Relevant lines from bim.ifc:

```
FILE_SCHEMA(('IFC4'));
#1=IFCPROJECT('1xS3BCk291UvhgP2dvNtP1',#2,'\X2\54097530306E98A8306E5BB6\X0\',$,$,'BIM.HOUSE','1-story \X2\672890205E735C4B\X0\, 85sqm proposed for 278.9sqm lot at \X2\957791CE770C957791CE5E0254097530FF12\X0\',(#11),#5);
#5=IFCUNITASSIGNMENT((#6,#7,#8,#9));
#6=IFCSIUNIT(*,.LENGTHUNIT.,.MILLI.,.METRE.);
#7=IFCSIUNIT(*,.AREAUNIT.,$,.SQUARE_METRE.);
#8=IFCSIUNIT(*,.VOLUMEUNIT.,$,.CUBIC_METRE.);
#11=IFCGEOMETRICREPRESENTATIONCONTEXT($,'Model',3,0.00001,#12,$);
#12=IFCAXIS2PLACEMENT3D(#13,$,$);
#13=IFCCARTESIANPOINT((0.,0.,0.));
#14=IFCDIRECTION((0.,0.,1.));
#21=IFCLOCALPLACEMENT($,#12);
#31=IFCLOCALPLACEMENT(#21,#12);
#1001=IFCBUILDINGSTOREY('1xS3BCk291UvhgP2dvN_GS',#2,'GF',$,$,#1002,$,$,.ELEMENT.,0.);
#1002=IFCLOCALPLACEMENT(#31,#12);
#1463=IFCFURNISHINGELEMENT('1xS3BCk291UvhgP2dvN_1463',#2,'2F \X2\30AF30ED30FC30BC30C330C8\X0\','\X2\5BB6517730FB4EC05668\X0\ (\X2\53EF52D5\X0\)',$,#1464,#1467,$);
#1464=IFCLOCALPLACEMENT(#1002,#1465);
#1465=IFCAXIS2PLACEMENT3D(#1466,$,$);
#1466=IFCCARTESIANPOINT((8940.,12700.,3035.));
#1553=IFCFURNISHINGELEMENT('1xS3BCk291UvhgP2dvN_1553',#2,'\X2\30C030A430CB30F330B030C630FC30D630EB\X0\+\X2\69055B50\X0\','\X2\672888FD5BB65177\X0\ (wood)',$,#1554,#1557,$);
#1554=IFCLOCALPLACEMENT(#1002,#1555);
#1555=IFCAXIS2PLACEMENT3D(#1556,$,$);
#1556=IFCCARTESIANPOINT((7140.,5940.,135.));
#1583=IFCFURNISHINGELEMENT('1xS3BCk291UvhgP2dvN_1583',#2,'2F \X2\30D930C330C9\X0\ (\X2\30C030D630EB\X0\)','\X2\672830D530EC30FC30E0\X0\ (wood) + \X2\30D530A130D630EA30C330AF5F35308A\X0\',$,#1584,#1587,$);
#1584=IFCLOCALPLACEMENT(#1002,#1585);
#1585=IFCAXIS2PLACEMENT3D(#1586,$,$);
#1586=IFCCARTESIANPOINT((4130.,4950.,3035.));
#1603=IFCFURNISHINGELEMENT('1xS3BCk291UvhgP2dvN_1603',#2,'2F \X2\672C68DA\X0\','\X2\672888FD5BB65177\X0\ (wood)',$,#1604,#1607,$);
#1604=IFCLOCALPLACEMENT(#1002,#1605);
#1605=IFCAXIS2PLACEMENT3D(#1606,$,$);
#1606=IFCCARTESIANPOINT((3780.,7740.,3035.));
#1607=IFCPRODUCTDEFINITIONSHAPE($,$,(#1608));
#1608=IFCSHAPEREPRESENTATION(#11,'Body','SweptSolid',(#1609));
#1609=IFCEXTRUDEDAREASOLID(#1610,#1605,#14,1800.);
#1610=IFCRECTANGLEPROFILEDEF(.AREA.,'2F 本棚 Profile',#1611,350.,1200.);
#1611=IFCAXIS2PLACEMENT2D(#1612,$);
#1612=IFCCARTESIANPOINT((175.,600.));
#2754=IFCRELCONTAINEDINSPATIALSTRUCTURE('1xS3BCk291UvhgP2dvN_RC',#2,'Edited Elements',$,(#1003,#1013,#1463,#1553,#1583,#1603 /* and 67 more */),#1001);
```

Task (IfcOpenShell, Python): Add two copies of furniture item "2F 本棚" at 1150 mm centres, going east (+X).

```python
import numpy as np
import ifcopenshell
import ifcopenshell.api.geometry
import ifcopenshell.api.root
import ifcopenshell.util.element
import ifcopenshell.util.placement
import ifcopenshell.util.unit

model = ifcopenshell.open("bim.ifc")
unit_scale = ifcopenshell.util.unit.calculate_unit_scale(model)


def reuse_history(source, copy):
    """copy_class also copies each property set's owner history, people and application; keep the originals."""
    for rel in copy.IsDefinedBy:
        if rel.is_a("IfcRelDefinesByProperties") and (history := rel.RelatingPropertyDefinition.OwnerHistory):
            rel.RelatingPropertyDefinition.OwnerHistory = source.OwnerHistory
            ifcopenshell.util.element.remove_deep2(model, history)


source = model.by_guid("1xS3BCk291UvhgP2dvN_1603")
base = ifcopenshell.util.placement.get_local_placement(source.ObjectPlacement)
step = np.array([1.0, 0.0, 0.0]) * 1.15 / unit_scale

for i in range(1, 3):
    copy = ifcopenshell.api.root.copy_class(model, product=source)
    copy.Representation = ifcopenshell.util.element.copy_deep(
        model, source.Representation, exclude=["IfcGeometricRepresentationContext", "IfcRepresentationMap"]
    )
    reuse_history(source, copy)
    matrix = base.copy()
    matrix[:3, 3] += i * step
    print("added at", matrix[:3, 3].round(3) + 0.0)
    ifcopenshell.api.geometry.edit_object_placement(model, product=copy, matrix=matrix, is_si=False)

model.write("bim-out.ifc")
```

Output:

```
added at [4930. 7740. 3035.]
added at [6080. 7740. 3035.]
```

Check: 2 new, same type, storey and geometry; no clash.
